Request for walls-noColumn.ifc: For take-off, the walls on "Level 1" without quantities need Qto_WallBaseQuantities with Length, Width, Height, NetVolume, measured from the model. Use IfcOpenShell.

First a look at what the model holds.

```python
import ifcopenshell
import ifcopenshell.util.element
import ifcopenshell.util.unit

model = ifcopenshell.open("walls-noColumn.ifc")
print(model.schema)
for unit_type in ("LENGTHUNIT", "AREAUNIT", "VOLUMEUNIT"):
    print(unit_type, ifcopenshell.util.unit.calculate_unit_scale(model, unit_type))
storey = next(s for s in model.by_type("IfcBuildingStorey") if s.Name == "Level 1")
walls = [e for e in ifcopenshell.util.element.get_decomposition(storey) if e.is_a("IfcWall")]
for e in sorted(walls, key=lambda e: e.id()):
    print(e.id(), e.is_a(), e.Name, list(ifcopenshell.util.element.get_psets(e, qtos_only=True)), sep=" | ")
```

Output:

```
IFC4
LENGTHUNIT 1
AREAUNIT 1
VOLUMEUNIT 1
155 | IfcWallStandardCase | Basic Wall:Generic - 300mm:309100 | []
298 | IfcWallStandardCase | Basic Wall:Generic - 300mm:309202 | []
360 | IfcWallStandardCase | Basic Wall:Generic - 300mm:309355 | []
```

```python
import ifcopenshell
import ifcopenshell.api.pset
import ifcopenshell.geom
import ifcopenshell.util.element
import ifcopenshell.util.shape
import ifcopenshell.util.unit

model = ifcopenshell.open("walls-noColumn.ifc")
unit_scale = ifcopenshell.util.unit.calculate_unit_scale(model)
volume_scale = ifcopenshell.util.unit.calculate_unit_scale(model, "VOLUMEUNIT")
settings = ifcopenshell.geom.settings()

storey = next(s for s in model.by_type("IfcBuildingStorey") if s.Name == "Level 1")
walls = [e for e in ifcopenshell.util.element.get_decomposition(storey) if e.is_a("IfcWall")]

for e in sorted(walls, key=lambda e: e.id()):
    if ifcopenshell.util.element.get_psets(e, qtos_only=True, should_inherit=False):
        continue
    # Geometry comes back in metres, in the element's own axes.
    shape = ifcopenshell.geom.create_shape(settings, e)
    values = {
        "Length": ifcopenshell.util.shape.get_x(shape.geometry) / unit_scale,
        "Width": ifcopenshell.util.shape.get_y(shape.geometry) / unit_scale,
        "Height": ifcopenshell.util.shape.get_z(shape.geometry) / unit_scale,
        "NetVolume": ifcopenshell.util.shape.get_volume(shape.geometry) / volume_scale,
    }
    qto = ifcopenshell.api.pset.add_qto(model, product=e, name="Qto_WallBaseQuantities")
    ifcopenshell.api.pset.edit_qto(model, qto=qto, properties=values)
    print(e.id(), {k: round(v, 3) for k, v in values.items()})

model.write("walls-noColumn_v2.ifc")
```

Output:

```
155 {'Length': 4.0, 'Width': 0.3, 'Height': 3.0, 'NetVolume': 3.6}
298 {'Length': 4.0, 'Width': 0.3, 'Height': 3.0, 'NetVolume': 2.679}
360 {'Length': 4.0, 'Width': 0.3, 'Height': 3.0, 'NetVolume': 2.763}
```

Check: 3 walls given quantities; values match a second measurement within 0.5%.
